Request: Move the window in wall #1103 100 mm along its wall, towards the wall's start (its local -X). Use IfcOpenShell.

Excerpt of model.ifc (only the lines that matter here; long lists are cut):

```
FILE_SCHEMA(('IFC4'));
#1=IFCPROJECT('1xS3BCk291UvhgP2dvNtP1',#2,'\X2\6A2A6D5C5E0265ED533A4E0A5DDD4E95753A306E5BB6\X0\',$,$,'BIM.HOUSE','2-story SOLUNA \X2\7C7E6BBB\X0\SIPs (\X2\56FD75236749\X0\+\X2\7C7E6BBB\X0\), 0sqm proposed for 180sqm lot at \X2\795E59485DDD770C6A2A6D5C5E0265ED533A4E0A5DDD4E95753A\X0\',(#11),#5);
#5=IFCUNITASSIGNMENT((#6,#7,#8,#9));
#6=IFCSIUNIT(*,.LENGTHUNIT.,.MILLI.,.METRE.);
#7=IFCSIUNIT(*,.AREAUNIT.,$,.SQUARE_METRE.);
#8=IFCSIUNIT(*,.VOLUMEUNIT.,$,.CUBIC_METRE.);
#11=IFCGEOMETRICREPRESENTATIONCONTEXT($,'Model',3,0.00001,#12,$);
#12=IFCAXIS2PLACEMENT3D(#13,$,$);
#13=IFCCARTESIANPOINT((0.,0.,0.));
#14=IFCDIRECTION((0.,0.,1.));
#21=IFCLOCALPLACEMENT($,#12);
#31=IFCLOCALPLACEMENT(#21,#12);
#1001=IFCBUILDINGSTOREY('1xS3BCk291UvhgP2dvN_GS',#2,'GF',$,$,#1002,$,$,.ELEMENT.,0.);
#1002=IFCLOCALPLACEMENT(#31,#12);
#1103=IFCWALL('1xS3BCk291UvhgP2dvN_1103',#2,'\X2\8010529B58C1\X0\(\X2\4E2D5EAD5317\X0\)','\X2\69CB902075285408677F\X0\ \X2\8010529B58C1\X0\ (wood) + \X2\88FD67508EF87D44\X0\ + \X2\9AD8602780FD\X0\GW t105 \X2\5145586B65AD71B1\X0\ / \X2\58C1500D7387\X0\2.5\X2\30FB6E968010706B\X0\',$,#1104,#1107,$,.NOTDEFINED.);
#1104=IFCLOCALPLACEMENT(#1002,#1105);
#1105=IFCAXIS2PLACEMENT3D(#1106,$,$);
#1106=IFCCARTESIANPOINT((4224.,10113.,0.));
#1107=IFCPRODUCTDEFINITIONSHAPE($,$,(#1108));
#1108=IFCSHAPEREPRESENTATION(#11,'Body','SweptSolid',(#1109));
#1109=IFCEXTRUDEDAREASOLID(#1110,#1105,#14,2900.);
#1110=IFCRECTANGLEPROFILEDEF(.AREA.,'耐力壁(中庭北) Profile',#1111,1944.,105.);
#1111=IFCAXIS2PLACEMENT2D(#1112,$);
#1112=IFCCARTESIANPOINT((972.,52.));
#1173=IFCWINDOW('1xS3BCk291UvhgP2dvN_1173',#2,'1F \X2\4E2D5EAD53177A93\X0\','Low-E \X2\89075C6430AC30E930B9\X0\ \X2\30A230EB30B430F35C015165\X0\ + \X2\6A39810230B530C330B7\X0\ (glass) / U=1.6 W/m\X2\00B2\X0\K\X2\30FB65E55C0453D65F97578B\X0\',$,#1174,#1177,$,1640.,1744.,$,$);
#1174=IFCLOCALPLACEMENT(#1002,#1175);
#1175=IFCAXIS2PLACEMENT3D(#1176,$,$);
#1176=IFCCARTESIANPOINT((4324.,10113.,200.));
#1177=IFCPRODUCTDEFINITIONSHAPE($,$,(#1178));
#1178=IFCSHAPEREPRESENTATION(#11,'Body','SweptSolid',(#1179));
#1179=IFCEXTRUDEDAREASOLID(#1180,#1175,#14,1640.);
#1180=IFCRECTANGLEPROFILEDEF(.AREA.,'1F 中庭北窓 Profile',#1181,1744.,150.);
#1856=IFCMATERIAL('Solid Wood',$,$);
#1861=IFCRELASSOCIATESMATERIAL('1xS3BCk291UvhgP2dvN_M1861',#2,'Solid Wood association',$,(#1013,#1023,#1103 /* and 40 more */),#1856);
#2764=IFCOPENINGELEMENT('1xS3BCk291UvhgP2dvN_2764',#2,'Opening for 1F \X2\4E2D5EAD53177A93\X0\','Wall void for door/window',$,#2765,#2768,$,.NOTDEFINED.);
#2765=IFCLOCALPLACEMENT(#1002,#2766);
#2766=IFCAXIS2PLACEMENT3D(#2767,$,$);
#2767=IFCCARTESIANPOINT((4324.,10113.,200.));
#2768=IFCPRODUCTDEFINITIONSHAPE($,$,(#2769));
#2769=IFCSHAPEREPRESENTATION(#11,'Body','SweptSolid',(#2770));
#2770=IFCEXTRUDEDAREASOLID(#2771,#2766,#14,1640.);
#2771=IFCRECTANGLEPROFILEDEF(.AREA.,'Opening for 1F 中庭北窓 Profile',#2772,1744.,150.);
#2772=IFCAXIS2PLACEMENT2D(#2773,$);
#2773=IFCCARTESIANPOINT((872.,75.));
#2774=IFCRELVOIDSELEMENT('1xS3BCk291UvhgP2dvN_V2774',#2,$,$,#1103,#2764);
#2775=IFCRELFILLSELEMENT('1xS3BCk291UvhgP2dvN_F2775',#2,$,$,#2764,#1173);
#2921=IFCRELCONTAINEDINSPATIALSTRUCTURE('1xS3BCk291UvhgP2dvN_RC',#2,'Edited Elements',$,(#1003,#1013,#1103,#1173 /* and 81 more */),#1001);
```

```python
import ifcopenshell
import ifcopenshell.api.geometry
import ifcopenshell.util.placement
import ifcopenshell.util.unit

model = ifcopenshell.open("model.ifc")
unit_scale = ifcopenshell.util.unit.calculate_unit_scale(model)

window = model.by_guid("1xS3BCk291UvhgP2dvN_1173")
opening = window.FillsVoids[0].RelatingOpeningElement
wall = opening.VoidsElements[0].RelatingBuildingElement

wall_matrix = ifcopenshell.util.placement.get_local_placement(wall.ObjectPlacement)
shift = wall_matrix[:3, 0] * -0.1 / unit_scale
before = ifcopenshell.util.placement.get_local_placement(window.ObjectPlacement)[:3, 3].copy()

# The window is not placed relative to its opening, so move both.
for product in (opening, window):
    matrix = ifcopenshell.util.placement.get_local_placement(product.ObjectPlacement)
    matrix[:3, 3] += shift
    ifcopenshell.api.geometry.edit_object_placement(model, product=product, matrix=matrix, is_si=False)

after = ifcopenshell.util.placement.get_local_placement(window.ObjectPlacement)[:3, 3]
print("window moved by", (after - before).round(3) + 0.0)

model.write("model_edited.ifc")
```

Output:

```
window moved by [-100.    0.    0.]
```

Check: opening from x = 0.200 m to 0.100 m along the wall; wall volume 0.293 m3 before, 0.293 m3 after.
